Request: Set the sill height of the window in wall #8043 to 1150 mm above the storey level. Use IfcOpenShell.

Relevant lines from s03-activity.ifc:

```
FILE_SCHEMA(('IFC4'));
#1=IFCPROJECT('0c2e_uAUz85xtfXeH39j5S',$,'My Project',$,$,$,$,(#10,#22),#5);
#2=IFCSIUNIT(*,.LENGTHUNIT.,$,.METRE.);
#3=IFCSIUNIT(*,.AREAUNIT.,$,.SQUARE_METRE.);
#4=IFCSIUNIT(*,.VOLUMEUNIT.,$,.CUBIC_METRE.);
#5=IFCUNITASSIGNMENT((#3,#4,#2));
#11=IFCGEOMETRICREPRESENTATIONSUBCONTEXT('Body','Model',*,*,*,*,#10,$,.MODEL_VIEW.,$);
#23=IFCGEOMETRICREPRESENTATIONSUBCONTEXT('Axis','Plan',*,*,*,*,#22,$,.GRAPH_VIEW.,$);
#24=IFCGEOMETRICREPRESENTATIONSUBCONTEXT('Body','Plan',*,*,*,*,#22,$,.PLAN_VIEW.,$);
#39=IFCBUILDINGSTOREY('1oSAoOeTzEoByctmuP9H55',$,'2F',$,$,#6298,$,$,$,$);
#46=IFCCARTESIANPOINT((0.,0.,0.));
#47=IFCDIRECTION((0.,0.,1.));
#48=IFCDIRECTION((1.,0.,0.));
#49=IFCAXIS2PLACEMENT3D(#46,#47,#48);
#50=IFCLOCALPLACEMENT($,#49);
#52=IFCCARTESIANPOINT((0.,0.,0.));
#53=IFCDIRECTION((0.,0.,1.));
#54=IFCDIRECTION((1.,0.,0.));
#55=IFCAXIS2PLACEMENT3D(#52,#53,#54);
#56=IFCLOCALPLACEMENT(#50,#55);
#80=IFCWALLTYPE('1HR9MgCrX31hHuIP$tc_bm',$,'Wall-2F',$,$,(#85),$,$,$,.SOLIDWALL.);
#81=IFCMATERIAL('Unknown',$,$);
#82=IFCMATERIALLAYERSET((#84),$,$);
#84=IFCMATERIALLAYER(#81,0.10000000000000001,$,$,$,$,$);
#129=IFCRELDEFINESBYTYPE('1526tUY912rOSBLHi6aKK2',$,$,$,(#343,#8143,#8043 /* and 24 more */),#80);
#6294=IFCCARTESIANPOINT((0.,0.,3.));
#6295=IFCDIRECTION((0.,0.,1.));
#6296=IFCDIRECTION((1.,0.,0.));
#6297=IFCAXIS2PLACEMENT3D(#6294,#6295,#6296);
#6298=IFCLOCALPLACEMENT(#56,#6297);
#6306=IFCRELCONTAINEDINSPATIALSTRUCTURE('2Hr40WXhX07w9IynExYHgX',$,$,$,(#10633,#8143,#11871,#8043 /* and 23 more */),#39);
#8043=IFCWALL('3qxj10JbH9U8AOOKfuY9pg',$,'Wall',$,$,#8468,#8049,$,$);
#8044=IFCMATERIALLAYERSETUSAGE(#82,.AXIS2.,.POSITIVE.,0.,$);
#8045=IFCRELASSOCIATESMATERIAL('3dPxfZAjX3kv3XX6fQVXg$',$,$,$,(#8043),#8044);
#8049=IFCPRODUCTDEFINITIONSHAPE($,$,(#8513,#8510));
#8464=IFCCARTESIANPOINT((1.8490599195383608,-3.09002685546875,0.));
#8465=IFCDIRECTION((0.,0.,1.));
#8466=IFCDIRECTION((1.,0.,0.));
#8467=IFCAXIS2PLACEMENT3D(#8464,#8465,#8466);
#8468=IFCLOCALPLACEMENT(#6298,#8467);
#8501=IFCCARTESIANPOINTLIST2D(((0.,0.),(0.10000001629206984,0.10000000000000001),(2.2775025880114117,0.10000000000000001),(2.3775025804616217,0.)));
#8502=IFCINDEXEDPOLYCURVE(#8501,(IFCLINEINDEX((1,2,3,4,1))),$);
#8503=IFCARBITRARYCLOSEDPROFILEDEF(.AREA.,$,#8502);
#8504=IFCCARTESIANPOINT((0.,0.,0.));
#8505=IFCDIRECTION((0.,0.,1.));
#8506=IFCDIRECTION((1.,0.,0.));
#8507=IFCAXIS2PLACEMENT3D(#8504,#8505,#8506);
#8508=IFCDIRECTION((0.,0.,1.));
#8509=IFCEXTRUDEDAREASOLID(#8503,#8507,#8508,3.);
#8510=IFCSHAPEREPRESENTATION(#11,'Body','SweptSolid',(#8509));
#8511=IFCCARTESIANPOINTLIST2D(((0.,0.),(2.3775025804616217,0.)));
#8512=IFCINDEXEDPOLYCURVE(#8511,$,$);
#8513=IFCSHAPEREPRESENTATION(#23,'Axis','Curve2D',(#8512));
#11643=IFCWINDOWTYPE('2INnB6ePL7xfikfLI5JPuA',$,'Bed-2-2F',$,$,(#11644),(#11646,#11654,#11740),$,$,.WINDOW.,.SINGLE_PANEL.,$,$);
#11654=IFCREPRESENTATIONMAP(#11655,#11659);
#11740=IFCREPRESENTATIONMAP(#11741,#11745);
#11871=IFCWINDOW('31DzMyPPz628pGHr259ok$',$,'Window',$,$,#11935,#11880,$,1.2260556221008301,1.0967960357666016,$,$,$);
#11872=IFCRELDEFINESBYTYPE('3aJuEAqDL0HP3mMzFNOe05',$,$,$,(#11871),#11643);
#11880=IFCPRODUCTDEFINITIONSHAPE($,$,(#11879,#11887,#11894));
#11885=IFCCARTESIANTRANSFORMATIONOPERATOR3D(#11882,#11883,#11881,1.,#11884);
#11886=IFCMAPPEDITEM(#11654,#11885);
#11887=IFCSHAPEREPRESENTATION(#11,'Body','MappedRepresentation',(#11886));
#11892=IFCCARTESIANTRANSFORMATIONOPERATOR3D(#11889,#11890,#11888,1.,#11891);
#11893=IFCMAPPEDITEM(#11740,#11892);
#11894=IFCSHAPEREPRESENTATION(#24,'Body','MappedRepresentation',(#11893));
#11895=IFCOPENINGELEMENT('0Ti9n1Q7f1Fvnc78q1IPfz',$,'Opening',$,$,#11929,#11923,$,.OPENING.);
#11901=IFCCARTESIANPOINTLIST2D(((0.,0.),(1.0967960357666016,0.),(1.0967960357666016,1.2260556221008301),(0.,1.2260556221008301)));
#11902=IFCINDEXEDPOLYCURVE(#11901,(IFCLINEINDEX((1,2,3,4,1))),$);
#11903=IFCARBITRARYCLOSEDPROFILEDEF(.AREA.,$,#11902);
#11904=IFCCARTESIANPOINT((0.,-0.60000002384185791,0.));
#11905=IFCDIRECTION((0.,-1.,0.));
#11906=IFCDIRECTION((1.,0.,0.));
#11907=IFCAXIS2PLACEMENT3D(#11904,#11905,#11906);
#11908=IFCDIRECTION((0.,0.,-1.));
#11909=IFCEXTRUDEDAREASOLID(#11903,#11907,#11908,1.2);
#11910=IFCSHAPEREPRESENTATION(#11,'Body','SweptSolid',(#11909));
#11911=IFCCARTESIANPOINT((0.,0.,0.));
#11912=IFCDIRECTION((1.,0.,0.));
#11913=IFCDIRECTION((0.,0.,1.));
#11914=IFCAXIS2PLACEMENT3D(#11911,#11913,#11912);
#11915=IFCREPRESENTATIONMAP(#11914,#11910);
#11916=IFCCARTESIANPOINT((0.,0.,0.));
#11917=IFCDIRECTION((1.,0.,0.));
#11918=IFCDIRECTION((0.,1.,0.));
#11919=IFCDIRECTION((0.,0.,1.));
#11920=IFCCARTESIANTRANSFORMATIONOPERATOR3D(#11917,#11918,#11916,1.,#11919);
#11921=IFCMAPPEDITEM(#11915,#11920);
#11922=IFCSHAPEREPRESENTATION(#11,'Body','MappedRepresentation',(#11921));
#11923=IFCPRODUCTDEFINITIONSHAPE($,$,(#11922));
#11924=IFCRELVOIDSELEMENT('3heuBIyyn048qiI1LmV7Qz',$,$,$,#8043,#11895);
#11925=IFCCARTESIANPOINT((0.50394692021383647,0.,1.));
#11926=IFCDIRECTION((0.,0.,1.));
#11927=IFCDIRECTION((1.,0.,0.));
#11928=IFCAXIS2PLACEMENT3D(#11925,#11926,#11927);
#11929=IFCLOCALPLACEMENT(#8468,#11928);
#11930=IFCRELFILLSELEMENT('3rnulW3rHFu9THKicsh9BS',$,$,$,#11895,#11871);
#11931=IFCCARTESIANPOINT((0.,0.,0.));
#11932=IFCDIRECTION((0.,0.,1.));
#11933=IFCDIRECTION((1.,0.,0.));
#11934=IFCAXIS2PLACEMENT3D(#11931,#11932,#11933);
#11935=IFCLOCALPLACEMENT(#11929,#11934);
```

```python
import numpy as np
import ifcopenshell
import ifcopenshell.api.geometry
import ifcopenshell.geom
import ifcopenshell.util.element
import ifcopenshell.util.placement
import ifcopenshell.util.shape
import ifcopenshell.util.unit

model = ifcopenshell.open("s03-activity.ifc")
unit_scale = ifcopenshell.util.unit.calculate_unit_scale(model)

window = model.by_guid("31DzMyPPz628pGHr259ok$")
opening = window.FillsVoids[0].RelatingOpeningElement
storey = ifcopenshell.util.element.get_container(window, ifc_class="IfcBuildingStorey")
level = ifcopenshell.util.placement.get_local_placement(storey.ObjectPlacement)[2, 3]

# The opening's origin need not be at the sill, so measure its lowest point.
shape = ifcopenshell.geom.create_shape(ifcopenshell.geom.settings(), opening)
bottom = ifcopenshell.util.shape.get_shape_bottom_elevation(shape, shape.geometry) / unit_scale
dz = level + 1.15 - bottom

shift = np.array([0.0, 0.0, dz])
# The window is placed relative to its opening, so it follows when the opening moves.
matrix = ifcopenshell.util.placement.get_local_placement(opening.ObjectPlacement)
matrix[:3, 3] += shift
ifcopenshell.api.geometry.edit_object_placement(
    model, product=opening, matrix=matrix, is_si=False, should_transform_children=True
)

print(f"moved by {dz * unit_scale:+.3f} m")

model.write("s03-activity_edited.ifc")
```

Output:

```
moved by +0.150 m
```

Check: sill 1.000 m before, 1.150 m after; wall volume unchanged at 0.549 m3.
